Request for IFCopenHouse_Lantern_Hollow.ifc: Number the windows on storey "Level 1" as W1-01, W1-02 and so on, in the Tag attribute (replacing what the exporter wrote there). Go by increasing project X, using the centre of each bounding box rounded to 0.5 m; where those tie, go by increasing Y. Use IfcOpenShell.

First a look at what the model holds.

```python
import ifcopenshell
import ifcopenshell.util.element
import ifcopenshell.util.placement

model = ifcopenshell.open("IFCopenHouse_Lantern_Hollow.ifc")
print(model.schema)
storey = next(s for s in model.by_type("IfcBuildingStorey") if s.Name == "Level 1")
windows = [e for e in ifcopenshell.util.element.get_decomposition(storey) if e.is_a("IfcWindow")]
for e in sorted(windows, key=lambda e: e.id()):
    origin = ifcopenshell.util.placement.get_local_placement(e.ObjectPlacement)[:3, 3]
    print(e.id(), e.Tag, e.Name, origin.round(2) + 0.0, sep=" | ")
```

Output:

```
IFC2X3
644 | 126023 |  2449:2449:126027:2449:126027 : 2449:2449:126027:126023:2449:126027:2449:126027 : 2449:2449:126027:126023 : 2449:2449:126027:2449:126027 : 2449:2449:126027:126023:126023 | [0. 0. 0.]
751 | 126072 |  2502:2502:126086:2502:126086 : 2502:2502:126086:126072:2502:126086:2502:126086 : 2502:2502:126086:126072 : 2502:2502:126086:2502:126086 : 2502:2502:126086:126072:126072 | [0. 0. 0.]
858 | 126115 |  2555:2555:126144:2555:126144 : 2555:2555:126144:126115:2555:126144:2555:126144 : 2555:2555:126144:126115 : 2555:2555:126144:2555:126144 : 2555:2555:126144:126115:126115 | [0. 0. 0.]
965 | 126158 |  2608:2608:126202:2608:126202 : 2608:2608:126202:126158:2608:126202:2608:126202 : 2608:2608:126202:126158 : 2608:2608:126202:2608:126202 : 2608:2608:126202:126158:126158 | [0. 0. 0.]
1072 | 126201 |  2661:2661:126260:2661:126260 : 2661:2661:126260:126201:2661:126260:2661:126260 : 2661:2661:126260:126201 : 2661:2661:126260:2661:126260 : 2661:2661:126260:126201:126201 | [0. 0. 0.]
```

```python
import ifcopenshell
import ifcopenshell.geom
import ifcopenshell.util.element
import ifcopenshell.util.shape

model = ifcopenshell.open("IFCopenHouse_Lantern_Hollow.ifc")
settings = ifcopenshell.geom.settings()
settings.set("use-world-coords", True)


def centre(element):
    shape = ifcopenshell.geom.create_shape(settings, element)
    return ifcopenshell.util.shape.get_bbox_centroid(shape.geometry)


storey = next(s for s in model.by_type("IfcBuildingStorey") if s.Name == "Level 1")
windows = [e for e in ifcopenshell.util.element.get_decomposition(storey) if e.is_a("IfcWindow")]

# Insertion points can sit at a corner or the storey origin, so sort by the geometry (in metres).
centres = {e: centre(e) for e in windows}
windows.sort(key=lambda e: (round(centres[e][0] / 0.5), centres[e][1]))

for i, e in enumerate(windows, start=1):
    number = f"W1-{i:02d}"
    e.Tag = number
    print(e.id(), number)

model.write("IFCopenHouse_Lantern_Hollow-out.ifc")
```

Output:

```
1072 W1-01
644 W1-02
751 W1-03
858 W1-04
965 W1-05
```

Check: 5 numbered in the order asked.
